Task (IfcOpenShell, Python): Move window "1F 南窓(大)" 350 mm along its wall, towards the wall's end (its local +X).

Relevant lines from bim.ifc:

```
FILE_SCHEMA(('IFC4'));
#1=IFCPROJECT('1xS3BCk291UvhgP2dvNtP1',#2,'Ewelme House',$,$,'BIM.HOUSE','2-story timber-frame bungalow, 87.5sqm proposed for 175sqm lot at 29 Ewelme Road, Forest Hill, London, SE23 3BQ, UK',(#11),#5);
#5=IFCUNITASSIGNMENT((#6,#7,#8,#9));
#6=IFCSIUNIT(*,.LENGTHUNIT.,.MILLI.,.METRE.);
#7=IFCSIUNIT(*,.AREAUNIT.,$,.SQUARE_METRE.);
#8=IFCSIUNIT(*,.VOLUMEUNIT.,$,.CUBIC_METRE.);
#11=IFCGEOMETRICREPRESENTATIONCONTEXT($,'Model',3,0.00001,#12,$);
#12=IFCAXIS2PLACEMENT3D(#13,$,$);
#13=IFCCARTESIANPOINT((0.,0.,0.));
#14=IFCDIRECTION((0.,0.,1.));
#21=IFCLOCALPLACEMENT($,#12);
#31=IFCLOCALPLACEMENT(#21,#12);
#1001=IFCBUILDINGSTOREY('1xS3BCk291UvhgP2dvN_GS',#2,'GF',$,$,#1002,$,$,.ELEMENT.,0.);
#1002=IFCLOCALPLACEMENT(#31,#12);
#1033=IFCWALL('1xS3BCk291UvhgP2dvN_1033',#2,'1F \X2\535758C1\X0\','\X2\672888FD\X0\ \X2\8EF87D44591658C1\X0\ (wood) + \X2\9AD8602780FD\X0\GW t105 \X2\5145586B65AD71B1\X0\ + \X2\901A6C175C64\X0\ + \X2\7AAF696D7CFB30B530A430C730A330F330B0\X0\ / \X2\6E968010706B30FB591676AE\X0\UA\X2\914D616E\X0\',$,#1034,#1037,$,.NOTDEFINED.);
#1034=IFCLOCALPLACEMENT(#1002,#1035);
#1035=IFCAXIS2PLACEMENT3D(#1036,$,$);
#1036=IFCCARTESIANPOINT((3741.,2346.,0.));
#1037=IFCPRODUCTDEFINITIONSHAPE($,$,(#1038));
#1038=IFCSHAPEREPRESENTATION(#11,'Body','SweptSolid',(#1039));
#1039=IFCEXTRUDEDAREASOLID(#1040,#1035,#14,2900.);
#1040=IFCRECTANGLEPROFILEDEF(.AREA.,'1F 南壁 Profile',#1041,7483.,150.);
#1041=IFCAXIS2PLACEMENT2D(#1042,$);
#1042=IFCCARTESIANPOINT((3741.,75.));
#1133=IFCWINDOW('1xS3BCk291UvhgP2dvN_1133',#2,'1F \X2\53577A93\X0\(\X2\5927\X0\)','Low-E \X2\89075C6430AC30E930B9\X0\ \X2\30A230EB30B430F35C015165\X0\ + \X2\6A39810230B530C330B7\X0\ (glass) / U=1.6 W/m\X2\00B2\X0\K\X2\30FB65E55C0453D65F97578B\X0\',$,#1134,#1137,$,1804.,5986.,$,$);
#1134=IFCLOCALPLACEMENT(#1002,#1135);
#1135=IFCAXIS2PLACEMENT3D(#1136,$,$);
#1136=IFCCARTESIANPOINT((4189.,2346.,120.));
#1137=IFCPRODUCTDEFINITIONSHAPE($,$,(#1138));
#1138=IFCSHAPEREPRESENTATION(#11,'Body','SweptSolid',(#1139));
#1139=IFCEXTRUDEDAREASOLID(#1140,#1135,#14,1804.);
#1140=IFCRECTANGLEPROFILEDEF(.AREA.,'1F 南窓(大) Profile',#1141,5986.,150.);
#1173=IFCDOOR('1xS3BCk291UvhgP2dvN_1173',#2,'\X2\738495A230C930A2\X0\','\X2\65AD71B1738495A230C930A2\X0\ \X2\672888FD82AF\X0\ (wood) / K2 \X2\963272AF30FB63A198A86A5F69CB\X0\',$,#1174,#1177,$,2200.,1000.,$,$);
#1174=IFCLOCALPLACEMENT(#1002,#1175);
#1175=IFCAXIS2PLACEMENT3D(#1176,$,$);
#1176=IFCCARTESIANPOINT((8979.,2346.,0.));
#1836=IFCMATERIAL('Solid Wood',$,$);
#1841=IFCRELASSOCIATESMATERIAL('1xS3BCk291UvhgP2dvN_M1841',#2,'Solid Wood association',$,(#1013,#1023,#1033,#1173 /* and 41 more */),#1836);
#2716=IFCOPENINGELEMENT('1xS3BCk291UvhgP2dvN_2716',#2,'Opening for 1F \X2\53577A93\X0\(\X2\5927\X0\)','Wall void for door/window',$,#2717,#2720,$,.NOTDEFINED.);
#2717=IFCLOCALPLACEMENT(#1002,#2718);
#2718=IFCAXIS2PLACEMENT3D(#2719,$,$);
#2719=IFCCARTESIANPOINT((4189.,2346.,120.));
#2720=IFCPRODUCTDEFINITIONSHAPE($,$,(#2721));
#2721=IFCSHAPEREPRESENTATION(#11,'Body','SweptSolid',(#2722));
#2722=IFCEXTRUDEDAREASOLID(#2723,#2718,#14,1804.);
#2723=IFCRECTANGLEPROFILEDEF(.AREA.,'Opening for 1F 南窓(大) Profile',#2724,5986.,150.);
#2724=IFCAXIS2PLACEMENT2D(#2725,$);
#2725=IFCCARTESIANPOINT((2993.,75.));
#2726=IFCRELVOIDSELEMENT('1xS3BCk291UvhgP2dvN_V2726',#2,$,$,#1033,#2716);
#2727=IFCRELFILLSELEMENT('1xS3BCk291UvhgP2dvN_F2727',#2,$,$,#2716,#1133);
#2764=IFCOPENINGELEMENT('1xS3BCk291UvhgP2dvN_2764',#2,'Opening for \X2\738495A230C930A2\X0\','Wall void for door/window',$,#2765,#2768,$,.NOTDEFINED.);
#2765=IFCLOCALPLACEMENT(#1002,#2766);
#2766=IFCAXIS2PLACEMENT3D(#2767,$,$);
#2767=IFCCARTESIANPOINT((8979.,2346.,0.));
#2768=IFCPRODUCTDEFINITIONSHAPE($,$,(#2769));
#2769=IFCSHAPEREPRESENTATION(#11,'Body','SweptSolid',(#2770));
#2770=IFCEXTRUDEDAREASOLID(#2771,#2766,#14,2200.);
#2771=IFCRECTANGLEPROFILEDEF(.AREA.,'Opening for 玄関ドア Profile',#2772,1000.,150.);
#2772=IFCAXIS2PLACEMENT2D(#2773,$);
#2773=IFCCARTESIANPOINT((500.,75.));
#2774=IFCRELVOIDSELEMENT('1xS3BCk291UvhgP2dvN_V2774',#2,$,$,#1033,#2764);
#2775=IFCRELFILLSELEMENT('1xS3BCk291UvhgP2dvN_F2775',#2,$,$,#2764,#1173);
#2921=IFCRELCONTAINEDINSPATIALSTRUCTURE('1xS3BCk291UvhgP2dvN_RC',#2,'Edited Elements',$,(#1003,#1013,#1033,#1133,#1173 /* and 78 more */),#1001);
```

```python
import ifcopenshell
import ifcopenshell.api.geometry
import ifcopenshell.util.placement

model = ifcopenshell.open("bim.ifc")

window = model.by_guid("1xS3BCk291UvhgP2dvN_1133")
opening = window.FillsVoids[0].RelatingOpeningElement
wall = opening.VoidsElements[0].RelatingBuildingElement

wall_matrix = ifcopenshell.util.placement.get_local_placement(wall.ObjectPlacement)
shift = wall_matrix[:3, 0] * 350.0
before = ifcopenshell.util.placement.get_local_placement(window.ObjectPlacement)[:3, 3].copy()

# The window is not placed relative to its opening, so move both.
for product in (opening, window):
    matrix = ifcopenshell.util.placement.get_local_placement(product.ObjectPlacement)
    matrix[:3, 3] += shift
    ifcopenshell.api.geometry.edit_object_placement(model, product=product, matrix=matrix, is_si=False)

after = ifcopenshell.util.placement.get_local_placement(window.ObjectPlacement)[:3, 3]
print("window moved by", (after - before).round(3) + 0.0)

model.write("bim_updated.ifc")
```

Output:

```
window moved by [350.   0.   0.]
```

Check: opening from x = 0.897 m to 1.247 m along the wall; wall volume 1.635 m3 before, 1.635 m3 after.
